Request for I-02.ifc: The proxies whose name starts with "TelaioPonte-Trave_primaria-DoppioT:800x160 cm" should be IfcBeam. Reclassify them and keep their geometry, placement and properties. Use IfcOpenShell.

First a look at what the model holds.

```python
import re

import ifcopenshell

model = ifcopenshell.open("I-02.ifc")
print(model.schema)
seen = {}
for e in model.by_type("IfcBuildingElementProxy"):
    name = re.sub(r":\d+(:\d+)?$", "", e.Name or "")  # drop the element id that some exporters append
    seen[name] = seen.get(name, 0) + 1
for name, count in sorted(seen.items()):
    print(count, "x", name)
```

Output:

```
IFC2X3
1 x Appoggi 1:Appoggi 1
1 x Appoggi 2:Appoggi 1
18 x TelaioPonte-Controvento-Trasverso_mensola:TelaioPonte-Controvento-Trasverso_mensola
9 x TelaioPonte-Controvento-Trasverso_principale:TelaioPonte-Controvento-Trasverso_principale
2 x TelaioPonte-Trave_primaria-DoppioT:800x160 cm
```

```python
import ifcopenshell
import ifcopenshell.api.root

model = ifcopenshell.open("I-02.ifc")

proxies = [e.id() for e in model.by_type("IfcBuildingElementProxy") if (e.Name or "").startswith("TelaioPonte-Trave_primaria-DoppioT:800x160 cm")]
for step_id in proxies:
    proxy = model.by_id(step_id)
    # Reclassifying a typed element also reclassifies its type and the type's other occurrences.
    if proxy.is_a("IfcBuildingElementProxy"):
        ifcopenshell.api.root.reassign_class(model, product=proxy, ifc_class="IfcBeam")

print(sum(model.by_id(i).is_a("IfcBeam") for i in proxies), "reclassified")

model.write("I-02_v2.ifc")
```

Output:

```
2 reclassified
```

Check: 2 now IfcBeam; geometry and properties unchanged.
